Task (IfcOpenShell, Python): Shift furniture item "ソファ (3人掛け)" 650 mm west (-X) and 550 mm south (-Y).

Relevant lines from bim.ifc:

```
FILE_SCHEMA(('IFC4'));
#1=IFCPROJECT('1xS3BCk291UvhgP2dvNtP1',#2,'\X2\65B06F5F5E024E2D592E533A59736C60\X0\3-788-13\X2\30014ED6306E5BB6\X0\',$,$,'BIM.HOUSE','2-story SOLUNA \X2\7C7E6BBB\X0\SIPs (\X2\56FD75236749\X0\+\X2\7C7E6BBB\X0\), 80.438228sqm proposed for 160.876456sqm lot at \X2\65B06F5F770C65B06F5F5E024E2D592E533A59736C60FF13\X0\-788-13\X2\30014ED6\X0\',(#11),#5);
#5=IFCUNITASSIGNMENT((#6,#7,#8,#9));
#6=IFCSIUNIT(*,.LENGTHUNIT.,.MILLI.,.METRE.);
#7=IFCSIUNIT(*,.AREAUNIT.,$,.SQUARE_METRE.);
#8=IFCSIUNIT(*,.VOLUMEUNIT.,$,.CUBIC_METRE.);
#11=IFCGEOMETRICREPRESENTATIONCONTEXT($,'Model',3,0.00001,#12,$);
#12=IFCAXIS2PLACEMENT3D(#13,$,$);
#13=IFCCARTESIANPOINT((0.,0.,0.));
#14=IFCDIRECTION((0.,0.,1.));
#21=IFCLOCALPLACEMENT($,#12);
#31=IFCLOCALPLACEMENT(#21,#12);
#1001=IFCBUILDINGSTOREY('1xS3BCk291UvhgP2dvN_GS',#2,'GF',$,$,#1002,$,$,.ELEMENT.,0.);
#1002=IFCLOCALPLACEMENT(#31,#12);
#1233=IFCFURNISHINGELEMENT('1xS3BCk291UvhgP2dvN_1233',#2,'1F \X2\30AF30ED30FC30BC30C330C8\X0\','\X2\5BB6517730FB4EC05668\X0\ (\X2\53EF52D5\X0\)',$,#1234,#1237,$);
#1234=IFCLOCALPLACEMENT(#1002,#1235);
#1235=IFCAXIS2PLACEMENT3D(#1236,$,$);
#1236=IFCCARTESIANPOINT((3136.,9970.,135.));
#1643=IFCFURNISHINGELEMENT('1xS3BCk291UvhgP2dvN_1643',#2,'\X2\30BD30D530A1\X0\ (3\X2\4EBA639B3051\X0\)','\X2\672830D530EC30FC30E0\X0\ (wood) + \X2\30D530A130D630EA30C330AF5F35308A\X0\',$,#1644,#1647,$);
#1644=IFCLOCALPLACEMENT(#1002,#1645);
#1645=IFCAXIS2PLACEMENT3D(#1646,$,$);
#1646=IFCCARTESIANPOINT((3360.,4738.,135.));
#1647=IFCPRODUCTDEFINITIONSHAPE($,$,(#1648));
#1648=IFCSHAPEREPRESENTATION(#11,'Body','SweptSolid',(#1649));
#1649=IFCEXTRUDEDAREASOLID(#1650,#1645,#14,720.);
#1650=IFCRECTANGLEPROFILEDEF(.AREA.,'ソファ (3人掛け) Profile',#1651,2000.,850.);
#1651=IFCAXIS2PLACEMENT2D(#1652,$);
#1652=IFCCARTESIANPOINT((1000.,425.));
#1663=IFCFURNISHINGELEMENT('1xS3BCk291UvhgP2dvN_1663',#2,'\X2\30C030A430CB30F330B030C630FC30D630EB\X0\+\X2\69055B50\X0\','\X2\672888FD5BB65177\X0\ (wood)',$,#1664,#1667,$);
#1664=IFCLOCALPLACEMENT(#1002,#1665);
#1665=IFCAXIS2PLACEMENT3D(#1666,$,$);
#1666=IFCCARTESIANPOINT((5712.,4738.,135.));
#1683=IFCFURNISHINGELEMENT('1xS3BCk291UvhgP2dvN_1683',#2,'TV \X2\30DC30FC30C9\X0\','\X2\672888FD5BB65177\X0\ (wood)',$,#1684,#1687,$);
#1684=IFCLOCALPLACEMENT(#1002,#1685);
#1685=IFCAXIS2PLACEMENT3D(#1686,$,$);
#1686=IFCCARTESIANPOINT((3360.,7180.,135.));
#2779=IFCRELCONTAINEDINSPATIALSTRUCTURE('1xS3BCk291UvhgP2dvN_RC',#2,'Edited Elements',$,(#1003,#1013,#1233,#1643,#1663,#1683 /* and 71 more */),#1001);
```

```python
import ifcopenshell
import ifcopenshell.api.geometry
import ifcopenshell.util.placement

model = ifcopenshell.open("bim.ifc")

item = model.by_guid("1xS3BCk291UvhgP2dvN_1643")
matrix = ifcopenshell.util.placement.get_local_placement(item.ObjectPlacement)
matrix[0, 3] -= 650.0
matrix[1, 3] -= 550.0
ifcopenshell.api.geometry.edit_object_placement(model, product=item, matrix=matrix, is_si=False)

print(ifcopenshell.util.placement.get_local_placement(item.ObjectPlacement).round(3) + 0.0)

model.write("bim_edited.ifc")
```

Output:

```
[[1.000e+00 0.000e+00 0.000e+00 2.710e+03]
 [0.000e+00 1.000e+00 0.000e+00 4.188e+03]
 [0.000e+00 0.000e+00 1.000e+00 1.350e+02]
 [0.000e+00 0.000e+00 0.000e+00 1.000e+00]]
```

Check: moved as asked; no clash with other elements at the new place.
